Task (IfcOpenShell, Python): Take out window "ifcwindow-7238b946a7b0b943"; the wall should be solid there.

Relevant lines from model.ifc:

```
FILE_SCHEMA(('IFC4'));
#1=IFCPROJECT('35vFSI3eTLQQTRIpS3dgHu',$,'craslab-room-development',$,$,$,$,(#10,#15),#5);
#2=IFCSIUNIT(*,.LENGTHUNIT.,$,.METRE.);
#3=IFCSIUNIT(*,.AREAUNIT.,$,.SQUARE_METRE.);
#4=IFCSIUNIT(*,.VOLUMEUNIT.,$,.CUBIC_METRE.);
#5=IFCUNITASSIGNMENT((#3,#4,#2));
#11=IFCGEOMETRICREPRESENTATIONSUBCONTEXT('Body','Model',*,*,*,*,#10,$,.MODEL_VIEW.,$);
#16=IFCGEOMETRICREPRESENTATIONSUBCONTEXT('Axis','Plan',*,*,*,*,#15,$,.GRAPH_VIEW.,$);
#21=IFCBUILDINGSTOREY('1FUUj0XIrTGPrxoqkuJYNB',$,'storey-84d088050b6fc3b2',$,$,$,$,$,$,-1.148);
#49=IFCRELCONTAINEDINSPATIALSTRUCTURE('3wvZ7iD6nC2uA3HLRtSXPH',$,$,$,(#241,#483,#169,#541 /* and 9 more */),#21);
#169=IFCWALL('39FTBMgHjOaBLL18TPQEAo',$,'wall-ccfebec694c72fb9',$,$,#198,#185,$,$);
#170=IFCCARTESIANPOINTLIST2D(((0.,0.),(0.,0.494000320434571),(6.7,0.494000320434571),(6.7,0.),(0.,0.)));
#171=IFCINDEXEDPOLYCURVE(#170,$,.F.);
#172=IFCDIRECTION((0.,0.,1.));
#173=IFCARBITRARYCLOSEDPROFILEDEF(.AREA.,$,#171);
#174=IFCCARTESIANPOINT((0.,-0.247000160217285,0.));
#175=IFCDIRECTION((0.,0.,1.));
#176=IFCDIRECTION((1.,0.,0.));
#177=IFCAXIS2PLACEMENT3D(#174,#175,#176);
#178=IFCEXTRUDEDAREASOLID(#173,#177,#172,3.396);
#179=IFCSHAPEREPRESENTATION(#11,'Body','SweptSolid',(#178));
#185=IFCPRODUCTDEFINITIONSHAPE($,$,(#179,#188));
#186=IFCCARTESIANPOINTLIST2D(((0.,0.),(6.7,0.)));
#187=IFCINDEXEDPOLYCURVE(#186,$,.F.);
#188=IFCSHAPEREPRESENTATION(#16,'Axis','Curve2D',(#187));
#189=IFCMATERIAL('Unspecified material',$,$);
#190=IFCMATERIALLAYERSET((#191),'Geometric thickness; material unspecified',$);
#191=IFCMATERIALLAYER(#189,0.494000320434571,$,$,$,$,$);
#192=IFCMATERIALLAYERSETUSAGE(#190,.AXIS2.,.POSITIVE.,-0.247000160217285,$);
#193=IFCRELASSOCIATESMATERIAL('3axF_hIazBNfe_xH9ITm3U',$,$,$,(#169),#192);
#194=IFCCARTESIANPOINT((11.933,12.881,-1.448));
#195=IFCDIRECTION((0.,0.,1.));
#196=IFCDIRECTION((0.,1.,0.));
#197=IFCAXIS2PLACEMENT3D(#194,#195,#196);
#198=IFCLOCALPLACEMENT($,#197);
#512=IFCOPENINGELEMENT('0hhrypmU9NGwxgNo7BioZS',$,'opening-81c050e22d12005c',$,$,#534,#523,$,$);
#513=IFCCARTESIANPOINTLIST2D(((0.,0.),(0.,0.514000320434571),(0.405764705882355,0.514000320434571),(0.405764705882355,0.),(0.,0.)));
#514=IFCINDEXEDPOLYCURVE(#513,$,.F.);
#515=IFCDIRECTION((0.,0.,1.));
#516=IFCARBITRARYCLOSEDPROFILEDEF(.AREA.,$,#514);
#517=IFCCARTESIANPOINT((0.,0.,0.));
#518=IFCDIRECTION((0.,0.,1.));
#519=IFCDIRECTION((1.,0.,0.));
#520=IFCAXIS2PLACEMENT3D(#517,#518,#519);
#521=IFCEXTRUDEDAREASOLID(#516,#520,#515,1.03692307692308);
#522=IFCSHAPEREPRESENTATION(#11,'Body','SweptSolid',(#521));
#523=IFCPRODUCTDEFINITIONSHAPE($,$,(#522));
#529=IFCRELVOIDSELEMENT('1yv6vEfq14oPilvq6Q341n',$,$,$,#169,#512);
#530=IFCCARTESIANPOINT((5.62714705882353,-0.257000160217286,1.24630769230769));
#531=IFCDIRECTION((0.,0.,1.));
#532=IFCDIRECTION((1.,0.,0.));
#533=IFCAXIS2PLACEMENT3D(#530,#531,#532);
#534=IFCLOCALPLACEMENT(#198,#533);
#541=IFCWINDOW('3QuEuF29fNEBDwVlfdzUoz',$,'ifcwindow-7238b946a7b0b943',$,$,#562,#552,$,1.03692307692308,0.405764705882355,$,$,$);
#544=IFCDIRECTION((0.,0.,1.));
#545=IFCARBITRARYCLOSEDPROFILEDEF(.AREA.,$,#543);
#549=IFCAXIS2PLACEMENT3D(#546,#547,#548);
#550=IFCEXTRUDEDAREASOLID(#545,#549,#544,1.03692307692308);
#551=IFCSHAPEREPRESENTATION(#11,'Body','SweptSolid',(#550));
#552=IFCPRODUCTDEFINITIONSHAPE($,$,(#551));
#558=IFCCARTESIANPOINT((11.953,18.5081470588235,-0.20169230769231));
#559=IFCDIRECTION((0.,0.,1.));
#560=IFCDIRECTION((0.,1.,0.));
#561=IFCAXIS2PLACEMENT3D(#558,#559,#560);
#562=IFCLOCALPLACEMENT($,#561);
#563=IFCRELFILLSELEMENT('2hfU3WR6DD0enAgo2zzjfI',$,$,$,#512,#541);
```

```python
import ifcopenshell
import ifcopenshell.api.feature
import ifcopenshell.api.root
import ifcopenshell.geom
import ifcopenshell.util.shape

model = ifcopenshell.open("model.ifc")
settings = ifcopenshell.geom.settings()


def volume(element):
    """Net volume in cubic metres, openings subtracted."""
    shape = ifcopenshell.geom.create_shape(settings, element)
    return ifcopenshell.util.shape.get_volume(shape.geometry)


window = model.by_id(541)
opening = window.FillsVoids[0].RelatingOpeningElement
wall = opening.VoidsElements[0].RelatingBuildingElement
before = volume(wall)

ifcopenshell.api.root.remove_product(model, product=window)
ifcopenshell.api.feature.remove_feature(model, feature=opening)

after = volume(wall)

print(f"wall volume {before:.3f} -> {after:.3f} m3")

model.write("model-out.ifc")
```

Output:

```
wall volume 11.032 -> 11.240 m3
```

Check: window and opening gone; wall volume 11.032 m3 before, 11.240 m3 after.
